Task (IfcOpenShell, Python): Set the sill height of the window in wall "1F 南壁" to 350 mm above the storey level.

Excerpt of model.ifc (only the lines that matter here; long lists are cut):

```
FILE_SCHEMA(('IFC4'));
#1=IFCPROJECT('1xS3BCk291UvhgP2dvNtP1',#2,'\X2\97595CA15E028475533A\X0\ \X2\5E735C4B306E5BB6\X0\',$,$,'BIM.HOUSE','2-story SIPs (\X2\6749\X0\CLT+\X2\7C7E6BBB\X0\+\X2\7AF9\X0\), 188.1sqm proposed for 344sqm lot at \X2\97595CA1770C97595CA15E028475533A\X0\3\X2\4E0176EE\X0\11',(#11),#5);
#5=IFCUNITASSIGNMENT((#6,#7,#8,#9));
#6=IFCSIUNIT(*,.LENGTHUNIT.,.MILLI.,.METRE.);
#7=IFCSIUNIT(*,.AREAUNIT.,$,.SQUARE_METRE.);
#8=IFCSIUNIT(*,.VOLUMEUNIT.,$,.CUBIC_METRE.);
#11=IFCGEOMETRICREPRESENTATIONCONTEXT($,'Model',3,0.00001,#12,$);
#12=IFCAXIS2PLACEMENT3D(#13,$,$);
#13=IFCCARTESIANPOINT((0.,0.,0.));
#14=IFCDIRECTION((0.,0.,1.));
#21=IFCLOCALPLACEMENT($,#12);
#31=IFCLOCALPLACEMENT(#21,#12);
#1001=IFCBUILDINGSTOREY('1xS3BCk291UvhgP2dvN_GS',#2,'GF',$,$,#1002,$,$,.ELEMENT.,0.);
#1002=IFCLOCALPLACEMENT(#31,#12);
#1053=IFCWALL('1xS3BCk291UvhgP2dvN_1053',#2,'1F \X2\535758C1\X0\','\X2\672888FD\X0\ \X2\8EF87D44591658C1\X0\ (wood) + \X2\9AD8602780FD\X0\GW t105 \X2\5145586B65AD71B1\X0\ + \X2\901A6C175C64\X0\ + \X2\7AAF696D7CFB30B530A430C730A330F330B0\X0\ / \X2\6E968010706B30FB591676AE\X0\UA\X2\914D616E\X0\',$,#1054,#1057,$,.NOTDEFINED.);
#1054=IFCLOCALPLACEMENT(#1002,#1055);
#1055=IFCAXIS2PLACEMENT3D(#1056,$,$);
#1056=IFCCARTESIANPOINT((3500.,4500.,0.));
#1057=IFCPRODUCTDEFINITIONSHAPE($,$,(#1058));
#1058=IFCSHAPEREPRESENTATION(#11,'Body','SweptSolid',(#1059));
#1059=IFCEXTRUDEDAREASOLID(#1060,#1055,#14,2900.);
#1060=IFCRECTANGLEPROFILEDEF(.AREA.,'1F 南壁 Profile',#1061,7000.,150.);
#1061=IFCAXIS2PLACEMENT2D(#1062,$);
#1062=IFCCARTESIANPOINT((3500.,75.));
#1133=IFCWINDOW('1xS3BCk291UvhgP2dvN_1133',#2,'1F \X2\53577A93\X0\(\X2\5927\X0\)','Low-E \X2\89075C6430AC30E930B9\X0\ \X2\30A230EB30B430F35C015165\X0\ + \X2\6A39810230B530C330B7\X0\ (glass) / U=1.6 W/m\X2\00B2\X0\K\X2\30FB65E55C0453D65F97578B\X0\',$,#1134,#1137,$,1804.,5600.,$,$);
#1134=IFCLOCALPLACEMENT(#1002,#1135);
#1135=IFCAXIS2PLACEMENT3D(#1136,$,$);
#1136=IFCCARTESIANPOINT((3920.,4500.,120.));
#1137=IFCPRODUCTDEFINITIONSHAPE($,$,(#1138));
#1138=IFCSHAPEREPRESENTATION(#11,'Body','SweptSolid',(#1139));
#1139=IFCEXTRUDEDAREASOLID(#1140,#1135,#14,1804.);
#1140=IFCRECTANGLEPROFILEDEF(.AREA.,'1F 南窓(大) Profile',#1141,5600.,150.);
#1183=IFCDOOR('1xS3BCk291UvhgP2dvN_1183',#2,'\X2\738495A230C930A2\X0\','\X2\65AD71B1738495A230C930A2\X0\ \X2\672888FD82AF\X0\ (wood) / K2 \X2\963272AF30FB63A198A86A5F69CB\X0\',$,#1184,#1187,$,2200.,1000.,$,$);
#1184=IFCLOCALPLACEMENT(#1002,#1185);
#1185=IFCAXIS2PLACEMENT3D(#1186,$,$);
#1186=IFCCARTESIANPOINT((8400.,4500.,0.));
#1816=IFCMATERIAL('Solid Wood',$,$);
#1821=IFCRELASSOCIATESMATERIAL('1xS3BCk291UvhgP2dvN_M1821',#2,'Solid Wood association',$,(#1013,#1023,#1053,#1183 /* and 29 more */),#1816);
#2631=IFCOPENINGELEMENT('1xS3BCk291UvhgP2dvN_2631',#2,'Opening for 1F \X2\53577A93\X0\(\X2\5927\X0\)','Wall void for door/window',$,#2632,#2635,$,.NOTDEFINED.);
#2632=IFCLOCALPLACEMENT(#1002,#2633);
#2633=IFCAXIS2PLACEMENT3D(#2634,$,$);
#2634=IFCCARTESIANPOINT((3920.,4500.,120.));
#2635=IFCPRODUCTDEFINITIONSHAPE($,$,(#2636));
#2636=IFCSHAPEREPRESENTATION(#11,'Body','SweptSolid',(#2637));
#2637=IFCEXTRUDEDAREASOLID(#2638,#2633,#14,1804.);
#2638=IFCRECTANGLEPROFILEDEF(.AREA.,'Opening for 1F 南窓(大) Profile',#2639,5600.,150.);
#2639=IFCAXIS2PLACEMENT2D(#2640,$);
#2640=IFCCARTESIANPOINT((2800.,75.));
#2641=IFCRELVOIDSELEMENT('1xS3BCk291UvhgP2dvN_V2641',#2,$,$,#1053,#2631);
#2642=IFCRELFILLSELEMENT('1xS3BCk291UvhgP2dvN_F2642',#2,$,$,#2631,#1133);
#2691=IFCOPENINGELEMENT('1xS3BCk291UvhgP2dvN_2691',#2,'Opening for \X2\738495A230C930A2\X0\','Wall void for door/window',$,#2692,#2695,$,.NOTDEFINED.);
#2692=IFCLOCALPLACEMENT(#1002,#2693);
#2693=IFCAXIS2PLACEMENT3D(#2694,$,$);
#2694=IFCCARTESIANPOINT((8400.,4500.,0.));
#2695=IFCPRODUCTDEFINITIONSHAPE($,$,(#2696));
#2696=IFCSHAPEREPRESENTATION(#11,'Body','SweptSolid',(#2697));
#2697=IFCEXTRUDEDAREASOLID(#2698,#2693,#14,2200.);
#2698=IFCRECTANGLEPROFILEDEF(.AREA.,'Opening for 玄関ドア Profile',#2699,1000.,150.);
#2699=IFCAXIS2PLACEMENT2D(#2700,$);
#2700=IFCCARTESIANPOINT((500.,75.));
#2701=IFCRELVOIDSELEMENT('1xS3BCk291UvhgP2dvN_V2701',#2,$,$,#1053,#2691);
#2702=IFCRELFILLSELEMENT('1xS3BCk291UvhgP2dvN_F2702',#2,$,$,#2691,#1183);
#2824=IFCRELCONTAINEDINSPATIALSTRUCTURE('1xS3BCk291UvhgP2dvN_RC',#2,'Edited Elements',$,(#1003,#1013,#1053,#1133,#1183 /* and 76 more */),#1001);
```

```python
import numpy as np
import ifcopenshell
import ifcopenshell.api.geometry
import ifcopenshell.geom
import ifcopenshell.util.element
import ifcopenshell.util.placement
import ifcopenshell.util.shape
import ifcopenshell.util.unit

model = ifcopenshell.open("model.ifc")
unit_scale = ifcopenshell.util.unit.calculate_unit_scale(model)

window = model.by_id(1133)
opening = window.FillsVoids[0].RelatingOpeningElement
storey = ifcopenshell.util.element.get_container(window, ifc_class="IfcBuildingStorey")
level = ifcopenshell.util.placement.get_local_placement(storey.ObjectPlacement)[2, 3]

# The opening's origin need not be at the sill, so measure its lowest point.
shape = ifcopenshell.geom.create_shape(ifcopenshell.geom.settings(), opening)
bottom = ifcopenshell.util.shape.get_shape_bottom_elevation(shape, shape.geometry) / unit_scale
dz = level + 0.35 / unit_scale - bottom

shift = np.array([0.0, 0.0, dz])
# The window is not placed relative to its opening, so move both.
for product in (opening, window):
    matrix = ifcopenshell.util.placement.get_local_placement(product.ObjectPlacement)
    matrix[:3, 3] += shift
    ifcopenshell.api.geometry.edit_object_placement(model, product=product, matrix=matrix, is_si=False)

print(f"moved by {dz * unit_scale:+.3f} m")

model.write("model_rev.ifc")
```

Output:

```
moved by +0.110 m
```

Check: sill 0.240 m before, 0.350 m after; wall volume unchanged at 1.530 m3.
